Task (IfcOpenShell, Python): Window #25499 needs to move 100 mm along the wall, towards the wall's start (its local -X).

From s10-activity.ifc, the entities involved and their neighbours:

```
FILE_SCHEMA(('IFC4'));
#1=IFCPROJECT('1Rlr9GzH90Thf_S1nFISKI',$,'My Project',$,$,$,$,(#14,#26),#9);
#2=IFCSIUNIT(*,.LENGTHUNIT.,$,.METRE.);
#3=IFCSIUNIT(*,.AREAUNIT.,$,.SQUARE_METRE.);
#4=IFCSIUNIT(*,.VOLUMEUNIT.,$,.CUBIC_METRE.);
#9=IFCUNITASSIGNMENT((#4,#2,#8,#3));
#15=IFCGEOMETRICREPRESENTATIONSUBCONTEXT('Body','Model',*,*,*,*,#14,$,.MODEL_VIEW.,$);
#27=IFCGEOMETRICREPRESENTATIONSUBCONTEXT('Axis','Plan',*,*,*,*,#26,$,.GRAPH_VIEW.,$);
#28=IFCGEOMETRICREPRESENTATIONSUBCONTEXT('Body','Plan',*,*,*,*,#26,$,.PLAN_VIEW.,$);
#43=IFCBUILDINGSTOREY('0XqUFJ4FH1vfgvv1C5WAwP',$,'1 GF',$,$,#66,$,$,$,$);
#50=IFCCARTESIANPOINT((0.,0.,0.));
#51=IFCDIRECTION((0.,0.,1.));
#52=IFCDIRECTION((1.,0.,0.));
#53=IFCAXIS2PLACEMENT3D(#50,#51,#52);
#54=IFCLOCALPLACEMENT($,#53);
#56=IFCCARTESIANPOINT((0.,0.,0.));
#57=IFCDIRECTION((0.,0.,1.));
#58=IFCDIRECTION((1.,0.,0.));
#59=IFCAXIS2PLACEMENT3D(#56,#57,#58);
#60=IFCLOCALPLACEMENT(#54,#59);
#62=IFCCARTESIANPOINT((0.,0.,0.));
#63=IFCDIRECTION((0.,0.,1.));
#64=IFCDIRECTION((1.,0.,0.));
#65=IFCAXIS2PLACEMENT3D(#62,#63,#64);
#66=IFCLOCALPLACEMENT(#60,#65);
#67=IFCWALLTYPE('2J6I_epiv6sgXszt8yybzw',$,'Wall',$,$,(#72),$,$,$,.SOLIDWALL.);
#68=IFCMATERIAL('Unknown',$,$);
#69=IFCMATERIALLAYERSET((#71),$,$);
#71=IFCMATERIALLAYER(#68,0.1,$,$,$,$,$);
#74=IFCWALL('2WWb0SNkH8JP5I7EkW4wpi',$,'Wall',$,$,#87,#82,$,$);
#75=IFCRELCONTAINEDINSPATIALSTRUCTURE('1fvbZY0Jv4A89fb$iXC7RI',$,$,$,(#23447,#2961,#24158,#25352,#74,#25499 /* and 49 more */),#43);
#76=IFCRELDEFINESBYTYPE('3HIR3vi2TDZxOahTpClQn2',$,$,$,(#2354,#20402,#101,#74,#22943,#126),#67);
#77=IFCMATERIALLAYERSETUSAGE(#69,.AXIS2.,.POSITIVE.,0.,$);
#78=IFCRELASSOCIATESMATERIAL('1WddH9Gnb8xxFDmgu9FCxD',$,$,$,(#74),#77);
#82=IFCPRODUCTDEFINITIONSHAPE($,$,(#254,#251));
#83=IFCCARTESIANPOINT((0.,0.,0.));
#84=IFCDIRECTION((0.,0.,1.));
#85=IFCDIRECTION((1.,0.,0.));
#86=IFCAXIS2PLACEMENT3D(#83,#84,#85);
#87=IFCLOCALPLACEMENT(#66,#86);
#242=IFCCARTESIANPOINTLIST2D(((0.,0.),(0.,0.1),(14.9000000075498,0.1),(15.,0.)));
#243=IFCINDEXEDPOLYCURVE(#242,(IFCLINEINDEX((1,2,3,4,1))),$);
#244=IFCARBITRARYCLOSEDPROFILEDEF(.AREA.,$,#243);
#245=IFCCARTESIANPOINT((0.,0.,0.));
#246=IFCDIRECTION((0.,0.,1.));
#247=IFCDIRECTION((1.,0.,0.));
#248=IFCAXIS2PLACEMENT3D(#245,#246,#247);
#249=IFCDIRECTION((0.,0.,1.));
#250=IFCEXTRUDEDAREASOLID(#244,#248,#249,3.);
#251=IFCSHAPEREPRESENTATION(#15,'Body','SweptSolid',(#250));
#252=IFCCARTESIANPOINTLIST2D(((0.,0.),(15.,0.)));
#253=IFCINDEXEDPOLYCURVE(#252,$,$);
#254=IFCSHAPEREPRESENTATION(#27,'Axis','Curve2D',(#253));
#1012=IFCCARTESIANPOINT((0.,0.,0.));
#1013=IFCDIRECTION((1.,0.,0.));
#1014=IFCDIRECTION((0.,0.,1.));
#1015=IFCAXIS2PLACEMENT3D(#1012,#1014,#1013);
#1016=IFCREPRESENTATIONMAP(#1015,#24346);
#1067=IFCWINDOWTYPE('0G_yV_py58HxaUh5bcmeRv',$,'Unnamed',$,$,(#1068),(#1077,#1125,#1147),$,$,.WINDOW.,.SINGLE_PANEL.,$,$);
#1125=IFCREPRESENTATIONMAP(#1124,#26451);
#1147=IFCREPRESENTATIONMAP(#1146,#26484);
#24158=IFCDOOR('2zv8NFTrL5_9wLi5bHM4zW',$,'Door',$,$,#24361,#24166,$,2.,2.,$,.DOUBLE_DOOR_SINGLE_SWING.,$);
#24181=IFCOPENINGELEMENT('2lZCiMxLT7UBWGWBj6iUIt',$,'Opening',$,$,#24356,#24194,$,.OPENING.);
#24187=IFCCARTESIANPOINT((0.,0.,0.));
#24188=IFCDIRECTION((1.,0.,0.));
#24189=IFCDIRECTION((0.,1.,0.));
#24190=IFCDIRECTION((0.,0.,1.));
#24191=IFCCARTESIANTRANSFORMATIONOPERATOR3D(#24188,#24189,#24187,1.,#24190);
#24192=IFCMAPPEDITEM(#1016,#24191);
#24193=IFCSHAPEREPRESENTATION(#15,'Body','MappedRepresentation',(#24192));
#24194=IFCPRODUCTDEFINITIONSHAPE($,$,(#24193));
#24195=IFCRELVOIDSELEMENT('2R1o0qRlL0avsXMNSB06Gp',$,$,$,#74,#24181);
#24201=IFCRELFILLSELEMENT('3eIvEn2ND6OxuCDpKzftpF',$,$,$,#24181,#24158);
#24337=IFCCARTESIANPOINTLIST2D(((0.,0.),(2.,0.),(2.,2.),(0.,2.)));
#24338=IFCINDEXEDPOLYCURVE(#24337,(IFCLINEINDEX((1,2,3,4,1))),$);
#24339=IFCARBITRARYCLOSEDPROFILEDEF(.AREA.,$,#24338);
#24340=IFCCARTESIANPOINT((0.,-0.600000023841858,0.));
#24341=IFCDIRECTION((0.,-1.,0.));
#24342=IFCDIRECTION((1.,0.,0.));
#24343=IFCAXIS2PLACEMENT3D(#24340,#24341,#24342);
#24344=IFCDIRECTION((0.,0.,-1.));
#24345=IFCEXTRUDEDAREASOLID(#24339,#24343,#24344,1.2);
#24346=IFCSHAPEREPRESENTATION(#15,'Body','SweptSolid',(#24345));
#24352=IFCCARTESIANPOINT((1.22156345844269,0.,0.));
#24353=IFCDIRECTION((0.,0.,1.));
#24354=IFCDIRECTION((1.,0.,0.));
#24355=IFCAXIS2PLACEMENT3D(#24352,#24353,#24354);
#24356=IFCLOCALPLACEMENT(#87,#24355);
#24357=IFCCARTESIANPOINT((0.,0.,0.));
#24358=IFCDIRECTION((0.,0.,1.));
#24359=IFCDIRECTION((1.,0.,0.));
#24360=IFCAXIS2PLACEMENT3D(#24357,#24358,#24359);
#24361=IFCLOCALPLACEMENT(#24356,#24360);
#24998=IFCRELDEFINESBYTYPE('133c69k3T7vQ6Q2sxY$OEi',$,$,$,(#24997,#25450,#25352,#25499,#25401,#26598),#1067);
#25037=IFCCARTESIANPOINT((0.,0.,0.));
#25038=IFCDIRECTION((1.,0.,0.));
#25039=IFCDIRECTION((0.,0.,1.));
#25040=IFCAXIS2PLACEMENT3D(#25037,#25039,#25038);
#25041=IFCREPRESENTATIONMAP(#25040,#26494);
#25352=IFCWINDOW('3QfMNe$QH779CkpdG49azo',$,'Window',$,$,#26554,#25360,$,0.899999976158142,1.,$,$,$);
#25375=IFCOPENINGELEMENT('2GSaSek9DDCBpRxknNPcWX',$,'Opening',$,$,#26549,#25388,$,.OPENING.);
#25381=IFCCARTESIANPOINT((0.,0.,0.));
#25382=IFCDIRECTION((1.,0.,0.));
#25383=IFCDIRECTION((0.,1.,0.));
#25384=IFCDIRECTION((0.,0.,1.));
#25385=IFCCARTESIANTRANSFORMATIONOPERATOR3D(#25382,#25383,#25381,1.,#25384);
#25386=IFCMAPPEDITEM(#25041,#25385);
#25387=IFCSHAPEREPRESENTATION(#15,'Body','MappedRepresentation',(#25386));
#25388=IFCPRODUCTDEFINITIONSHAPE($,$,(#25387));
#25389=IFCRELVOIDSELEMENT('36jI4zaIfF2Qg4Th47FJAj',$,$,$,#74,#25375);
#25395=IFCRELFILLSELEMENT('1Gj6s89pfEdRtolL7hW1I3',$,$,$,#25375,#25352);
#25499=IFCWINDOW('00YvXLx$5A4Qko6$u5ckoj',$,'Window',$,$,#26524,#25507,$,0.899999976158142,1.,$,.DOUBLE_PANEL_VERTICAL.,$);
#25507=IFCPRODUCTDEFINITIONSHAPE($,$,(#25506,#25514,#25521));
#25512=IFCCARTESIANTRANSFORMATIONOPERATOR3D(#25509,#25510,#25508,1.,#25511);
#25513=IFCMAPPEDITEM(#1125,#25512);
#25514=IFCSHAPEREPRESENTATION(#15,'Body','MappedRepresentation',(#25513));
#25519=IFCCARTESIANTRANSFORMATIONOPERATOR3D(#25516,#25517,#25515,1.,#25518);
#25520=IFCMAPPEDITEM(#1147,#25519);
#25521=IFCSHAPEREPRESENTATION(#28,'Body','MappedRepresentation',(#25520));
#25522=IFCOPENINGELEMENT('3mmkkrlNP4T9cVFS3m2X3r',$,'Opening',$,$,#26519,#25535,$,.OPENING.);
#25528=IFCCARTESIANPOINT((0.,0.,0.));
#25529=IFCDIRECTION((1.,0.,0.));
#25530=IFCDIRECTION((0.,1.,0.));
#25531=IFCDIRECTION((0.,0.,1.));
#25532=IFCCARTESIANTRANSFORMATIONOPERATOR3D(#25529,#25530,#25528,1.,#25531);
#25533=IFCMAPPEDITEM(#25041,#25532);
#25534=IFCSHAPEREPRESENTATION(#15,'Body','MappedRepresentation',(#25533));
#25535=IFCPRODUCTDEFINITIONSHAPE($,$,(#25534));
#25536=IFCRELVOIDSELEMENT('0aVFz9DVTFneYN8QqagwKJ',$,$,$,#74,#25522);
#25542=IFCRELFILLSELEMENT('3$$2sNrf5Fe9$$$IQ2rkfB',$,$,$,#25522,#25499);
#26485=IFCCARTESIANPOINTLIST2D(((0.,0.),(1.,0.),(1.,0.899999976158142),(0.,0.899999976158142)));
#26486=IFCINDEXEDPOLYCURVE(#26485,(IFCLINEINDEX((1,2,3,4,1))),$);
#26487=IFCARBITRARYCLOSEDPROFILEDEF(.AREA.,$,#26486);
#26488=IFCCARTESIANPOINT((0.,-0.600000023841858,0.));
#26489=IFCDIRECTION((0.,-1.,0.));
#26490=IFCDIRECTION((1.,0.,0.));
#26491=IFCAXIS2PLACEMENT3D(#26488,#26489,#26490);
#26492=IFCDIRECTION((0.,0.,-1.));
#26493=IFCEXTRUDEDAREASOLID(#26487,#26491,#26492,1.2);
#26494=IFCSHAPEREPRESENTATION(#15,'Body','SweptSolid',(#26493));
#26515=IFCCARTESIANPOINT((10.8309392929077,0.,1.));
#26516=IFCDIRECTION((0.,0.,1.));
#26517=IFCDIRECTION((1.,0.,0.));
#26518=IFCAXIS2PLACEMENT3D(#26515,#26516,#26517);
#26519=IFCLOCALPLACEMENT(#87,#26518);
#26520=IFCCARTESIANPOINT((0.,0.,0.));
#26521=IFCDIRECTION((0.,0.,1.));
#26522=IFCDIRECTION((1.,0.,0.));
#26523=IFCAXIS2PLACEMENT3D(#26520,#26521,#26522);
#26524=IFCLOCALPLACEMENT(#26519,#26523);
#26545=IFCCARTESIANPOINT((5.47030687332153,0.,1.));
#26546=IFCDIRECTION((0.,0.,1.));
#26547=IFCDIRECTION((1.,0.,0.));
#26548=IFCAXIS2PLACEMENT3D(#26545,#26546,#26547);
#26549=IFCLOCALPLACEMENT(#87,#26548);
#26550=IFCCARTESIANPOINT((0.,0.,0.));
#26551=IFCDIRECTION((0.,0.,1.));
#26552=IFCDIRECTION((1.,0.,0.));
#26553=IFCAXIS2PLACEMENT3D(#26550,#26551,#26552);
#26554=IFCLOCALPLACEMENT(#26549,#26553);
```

```python
import ifcopenshell
import ifcopenshell.api.geometry
import ifcopenshell.util.placement
import ifcopenshell.util.unit

model = ifcopenshell.open("s10-activity.ifc")
unit_scale = ifcopenshell.util.unit.calculate_unit_scale(model)

window = model.by_id(25499)
opening = window.FillsVoids[0].RelatingOpeningElement
wall = opening.VoidsElements[0].RelatingBuildingElement

wall_matrix = ifcopenshell.util.placement.get_local_placement(wall.ObjectPlacement)
shift = wall_matrix[:3, 0] * -0.1 / unit_scale
before = ifcopenshell.util.placement.get_local_placement(window.ObjectPlacement)[:3, 3].copy()

# The window is placed relative to its opening, so it follows when the opening moves.
matrix = ifcopenshell.util.placement.get_local_placement(opening.ObjectPlacement)
matrix[:3, 3] += shift
ifcopenshell.api.geometry.edit_object_placement(
    model, product=opening, matrix=matrix, is_si=False, should_transform_children=True
)

after = ifcopenshell.util.placement.get_local_placement(window.ObjectPlacement)[:3, 3]
print("window moved by", (after - before).round(3) + 0.0)

model.write("s10-activity-out.ifc")
```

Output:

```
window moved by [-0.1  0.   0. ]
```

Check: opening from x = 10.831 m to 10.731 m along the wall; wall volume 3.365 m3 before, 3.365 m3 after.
